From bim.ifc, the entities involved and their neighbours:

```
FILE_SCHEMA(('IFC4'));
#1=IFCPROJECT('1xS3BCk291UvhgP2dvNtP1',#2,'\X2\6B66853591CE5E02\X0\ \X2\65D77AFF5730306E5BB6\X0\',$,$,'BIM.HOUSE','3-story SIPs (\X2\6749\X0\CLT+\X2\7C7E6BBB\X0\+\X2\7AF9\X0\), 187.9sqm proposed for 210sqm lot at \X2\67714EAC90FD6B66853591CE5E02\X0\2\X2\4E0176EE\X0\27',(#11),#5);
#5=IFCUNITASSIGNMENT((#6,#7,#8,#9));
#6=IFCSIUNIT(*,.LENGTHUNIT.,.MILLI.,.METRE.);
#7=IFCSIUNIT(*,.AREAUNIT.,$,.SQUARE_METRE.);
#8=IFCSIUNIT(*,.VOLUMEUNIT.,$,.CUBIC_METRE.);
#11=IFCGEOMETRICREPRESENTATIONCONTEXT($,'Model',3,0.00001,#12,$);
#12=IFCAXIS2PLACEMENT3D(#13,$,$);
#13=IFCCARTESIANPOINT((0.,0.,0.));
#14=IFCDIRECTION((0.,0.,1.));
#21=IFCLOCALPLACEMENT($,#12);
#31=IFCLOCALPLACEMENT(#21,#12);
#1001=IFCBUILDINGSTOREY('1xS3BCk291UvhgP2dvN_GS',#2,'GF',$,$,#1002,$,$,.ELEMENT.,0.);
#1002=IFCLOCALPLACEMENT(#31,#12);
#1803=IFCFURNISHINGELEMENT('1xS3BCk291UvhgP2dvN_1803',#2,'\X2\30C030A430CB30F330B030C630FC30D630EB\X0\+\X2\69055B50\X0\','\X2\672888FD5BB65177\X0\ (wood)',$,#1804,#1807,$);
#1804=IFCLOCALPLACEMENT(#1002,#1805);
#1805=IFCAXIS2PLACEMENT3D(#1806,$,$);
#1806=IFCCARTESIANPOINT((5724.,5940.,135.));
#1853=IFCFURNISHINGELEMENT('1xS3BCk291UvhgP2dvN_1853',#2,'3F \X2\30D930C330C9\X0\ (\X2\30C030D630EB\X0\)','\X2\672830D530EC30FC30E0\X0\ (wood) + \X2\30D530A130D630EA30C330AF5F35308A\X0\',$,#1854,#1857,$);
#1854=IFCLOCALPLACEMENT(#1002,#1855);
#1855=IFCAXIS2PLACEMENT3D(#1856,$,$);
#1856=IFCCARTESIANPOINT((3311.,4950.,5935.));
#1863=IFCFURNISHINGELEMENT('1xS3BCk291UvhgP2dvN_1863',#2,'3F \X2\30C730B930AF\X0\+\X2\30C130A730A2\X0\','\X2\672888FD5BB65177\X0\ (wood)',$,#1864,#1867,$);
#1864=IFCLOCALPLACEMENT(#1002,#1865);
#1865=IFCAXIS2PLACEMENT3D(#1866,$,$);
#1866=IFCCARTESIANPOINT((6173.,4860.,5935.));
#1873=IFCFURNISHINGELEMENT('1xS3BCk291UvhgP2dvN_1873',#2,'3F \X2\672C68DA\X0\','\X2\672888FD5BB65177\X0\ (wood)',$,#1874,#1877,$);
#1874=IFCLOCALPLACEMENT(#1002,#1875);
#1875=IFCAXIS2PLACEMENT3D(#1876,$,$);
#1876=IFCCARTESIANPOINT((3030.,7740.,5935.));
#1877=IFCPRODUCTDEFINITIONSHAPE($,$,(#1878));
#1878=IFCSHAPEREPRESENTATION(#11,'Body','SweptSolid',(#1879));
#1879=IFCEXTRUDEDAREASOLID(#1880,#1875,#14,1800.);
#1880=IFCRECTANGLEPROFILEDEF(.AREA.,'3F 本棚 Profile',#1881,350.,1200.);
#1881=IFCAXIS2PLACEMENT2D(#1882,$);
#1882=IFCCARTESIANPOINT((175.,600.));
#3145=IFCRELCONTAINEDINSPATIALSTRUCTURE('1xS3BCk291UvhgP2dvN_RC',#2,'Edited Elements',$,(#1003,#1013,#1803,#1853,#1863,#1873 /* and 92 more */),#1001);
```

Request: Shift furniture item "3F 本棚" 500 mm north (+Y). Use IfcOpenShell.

```python
import ifcopenshell
import ifcopenshell.api.geometry
import ifcopenshell.util.placement

model = ifcopenshell.open("bim.ifc")

item = model.by_id(1873)
matrix = ifcopenshell.util.placement.get_local_placement(item.ObjectPlacement)
matrix[1, 3] += 500.0
ifcopenshell.api.geometry.edit_object_placement(model, product=item, matrix=matrix, is_si=False)

print(ifcopenshell.util.placement.get_local_placement(item.ObjectPlacement).round(3) + 0.0)

model.write("bim_updated.ifc")
```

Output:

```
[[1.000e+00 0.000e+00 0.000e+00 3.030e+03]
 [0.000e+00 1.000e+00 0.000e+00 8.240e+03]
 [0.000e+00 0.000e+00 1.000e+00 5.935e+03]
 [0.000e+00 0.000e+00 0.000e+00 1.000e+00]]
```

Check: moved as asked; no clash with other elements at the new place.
